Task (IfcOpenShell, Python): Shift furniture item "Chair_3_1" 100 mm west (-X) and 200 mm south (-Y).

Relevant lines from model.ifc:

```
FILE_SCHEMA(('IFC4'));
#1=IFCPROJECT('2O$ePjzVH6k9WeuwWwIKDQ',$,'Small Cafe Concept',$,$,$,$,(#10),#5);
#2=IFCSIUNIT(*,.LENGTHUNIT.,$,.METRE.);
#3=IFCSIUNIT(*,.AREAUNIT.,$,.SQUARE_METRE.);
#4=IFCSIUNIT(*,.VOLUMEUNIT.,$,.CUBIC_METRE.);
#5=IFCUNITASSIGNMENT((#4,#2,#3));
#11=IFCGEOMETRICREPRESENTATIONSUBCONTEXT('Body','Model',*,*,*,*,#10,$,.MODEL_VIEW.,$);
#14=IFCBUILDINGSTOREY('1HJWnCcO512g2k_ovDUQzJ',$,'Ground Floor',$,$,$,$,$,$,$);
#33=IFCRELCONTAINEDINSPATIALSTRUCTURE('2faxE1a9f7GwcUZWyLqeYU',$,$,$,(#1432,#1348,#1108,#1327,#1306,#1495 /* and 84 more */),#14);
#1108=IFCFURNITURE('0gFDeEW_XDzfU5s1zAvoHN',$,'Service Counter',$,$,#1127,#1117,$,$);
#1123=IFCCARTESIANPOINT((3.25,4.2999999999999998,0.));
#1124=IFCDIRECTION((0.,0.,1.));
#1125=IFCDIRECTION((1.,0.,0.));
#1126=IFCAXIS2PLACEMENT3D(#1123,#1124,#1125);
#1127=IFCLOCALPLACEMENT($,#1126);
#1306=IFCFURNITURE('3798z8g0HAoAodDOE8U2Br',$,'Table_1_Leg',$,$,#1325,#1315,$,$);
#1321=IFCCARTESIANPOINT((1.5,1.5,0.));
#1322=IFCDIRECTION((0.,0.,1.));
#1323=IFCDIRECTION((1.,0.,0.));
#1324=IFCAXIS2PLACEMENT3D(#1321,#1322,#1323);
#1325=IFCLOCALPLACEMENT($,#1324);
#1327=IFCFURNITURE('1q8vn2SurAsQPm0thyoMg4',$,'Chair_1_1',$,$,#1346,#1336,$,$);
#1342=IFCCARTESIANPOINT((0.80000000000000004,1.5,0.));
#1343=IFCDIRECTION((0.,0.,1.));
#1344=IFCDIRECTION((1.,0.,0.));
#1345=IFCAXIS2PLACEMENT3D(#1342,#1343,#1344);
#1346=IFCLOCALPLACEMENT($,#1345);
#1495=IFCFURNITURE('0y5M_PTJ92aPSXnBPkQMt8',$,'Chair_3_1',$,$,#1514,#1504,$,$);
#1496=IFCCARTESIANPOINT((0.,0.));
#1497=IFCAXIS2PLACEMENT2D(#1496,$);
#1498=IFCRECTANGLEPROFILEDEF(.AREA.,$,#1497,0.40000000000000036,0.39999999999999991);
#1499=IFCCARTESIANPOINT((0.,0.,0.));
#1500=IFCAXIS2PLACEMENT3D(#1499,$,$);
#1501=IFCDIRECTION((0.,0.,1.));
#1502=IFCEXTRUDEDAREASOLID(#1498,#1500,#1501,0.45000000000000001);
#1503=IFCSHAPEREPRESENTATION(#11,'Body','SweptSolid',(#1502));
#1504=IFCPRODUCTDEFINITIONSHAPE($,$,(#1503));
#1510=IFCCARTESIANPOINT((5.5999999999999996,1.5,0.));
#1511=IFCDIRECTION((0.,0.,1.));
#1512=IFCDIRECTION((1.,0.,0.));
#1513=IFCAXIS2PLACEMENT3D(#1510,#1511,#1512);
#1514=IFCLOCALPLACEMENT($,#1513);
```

```python
import ifcopenshell
import ifcopenshell.api.geometry
import ifcopenshell.util.placement
import ifcopenshell.util.unit

model = ifcopenshell.open("model.ifc")
unit_scale = ifcopenshell.util.unit.calculate_unit_scale(model)

item = model.by_guid("0y5M_PTJ92aPSXnBPkQMt8")
matrix = ifcopenshell.util.placement.get_local_placement(item.ObjectPlacement)
matrix[0, 3] -= 0.1 / unit_scale
matrix[1, 3] -= 0.2 / unit_scale
ifcopenshell.api.geometry.edit_object_placement(model, product=item, matrix=matrix, is_si=False)

print(ifcopenshell.util.placement.get_local_placement(item.ObjectPlacement).round(3) + 0.0)

model.write("model-out.ifc")
```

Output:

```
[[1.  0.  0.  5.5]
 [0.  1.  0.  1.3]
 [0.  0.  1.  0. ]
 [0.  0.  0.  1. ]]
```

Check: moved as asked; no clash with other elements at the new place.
